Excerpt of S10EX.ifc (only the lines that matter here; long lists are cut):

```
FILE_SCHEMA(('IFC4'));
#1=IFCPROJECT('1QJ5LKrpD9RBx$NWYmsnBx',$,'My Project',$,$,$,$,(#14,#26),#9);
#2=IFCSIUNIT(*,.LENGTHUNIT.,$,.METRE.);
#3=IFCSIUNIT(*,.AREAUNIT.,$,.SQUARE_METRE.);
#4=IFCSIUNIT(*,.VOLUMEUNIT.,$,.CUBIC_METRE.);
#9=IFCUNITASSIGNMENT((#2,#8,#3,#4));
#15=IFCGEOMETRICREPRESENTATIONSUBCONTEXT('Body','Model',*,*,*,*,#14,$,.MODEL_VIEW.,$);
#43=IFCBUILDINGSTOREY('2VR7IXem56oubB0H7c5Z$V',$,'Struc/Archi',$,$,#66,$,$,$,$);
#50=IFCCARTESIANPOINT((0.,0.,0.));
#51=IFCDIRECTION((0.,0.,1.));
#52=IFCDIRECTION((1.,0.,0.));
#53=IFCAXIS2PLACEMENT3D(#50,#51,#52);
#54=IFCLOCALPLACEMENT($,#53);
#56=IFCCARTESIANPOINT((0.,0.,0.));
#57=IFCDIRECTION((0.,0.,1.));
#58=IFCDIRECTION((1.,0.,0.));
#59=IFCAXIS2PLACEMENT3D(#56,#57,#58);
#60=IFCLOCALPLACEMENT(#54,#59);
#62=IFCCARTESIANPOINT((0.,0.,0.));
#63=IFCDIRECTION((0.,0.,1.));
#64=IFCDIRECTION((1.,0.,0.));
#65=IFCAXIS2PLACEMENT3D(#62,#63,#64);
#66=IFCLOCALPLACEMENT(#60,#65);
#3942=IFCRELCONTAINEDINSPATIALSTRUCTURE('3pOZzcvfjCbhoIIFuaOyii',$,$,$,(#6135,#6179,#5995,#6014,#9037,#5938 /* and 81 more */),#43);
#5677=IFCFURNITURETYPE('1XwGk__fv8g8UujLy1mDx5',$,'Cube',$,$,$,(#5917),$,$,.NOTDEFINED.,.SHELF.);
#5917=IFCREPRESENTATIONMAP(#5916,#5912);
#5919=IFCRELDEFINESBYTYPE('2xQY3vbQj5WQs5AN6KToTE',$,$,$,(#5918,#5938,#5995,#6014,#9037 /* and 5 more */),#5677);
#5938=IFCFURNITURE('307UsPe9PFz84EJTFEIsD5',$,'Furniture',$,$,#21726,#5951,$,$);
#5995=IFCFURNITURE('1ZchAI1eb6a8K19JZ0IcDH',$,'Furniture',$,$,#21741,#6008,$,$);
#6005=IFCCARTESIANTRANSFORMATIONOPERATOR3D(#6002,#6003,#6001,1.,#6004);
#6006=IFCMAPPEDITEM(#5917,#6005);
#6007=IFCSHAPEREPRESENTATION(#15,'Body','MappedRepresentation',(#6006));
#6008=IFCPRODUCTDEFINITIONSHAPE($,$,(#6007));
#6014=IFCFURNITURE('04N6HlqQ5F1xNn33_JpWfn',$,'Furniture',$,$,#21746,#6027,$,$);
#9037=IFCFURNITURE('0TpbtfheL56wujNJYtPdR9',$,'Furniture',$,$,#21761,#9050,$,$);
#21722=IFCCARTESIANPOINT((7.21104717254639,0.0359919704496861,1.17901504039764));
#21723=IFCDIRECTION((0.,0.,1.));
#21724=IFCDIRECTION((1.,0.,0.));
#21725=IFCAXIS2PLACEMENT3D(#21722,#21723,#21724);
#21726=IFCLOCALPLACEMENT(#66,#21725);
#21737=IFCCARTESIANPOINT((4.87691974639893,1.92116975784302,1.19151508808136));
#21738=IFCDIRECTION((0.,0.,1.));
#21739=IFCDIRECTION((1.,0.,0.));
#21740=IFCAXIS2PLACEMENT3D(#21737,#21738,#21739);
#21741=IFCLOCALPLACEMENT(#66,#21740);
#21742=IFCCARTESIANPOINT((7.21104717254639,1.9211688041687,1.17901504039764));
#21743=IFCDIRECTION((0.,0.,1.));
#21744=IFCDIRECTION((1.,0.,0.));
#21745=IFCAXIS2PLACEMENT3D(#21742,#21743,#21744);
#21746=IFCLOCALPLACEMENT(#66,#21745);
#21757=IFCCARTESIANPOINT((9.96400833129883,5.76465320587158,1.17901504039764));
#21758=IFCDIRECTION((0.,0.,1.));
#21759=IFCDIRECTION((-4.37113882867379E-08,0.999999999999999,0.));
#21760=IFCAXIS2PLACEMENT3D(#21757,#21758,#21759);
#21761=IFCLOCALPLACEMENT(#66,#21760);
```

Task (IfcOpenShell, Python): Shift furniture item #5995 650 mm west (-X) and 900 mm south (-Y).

```python
import ifcopenshell
import ifcopenshell.api.geometry
import ifcopenshell.util.placement
import ifcopenshell.util.unit

model = ifcopenshell.open("S10EX.ifc")
unit_scale = ifcopenshell.util.unit.calculate_unit_scale(model)

item = model.by_guid("1ZchAI1eb6a8K19JZ0IcDH")
matrix = ifcopenshell.util.placement.get_local_placement(item.ObjectPlacement)
matrix[0, 3] -= 0.65 / unit_scale
matrix[1, 3] -= 0.9 / unit_scale
ifcopenshell.api.geometry.edit_object_placement(model, product=item, matrix=matrix, is_si=False)

print(ifcopenshell.util.placement.get_local_placement(item.ObjectPlacement).round(3) + 0.0)

model.write("S10EX_v2.ifc")
```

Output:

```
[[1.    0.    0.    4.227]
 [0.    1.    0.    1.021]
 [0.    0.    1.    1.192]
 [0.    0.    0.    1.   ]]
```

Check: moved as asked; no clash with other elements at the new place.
